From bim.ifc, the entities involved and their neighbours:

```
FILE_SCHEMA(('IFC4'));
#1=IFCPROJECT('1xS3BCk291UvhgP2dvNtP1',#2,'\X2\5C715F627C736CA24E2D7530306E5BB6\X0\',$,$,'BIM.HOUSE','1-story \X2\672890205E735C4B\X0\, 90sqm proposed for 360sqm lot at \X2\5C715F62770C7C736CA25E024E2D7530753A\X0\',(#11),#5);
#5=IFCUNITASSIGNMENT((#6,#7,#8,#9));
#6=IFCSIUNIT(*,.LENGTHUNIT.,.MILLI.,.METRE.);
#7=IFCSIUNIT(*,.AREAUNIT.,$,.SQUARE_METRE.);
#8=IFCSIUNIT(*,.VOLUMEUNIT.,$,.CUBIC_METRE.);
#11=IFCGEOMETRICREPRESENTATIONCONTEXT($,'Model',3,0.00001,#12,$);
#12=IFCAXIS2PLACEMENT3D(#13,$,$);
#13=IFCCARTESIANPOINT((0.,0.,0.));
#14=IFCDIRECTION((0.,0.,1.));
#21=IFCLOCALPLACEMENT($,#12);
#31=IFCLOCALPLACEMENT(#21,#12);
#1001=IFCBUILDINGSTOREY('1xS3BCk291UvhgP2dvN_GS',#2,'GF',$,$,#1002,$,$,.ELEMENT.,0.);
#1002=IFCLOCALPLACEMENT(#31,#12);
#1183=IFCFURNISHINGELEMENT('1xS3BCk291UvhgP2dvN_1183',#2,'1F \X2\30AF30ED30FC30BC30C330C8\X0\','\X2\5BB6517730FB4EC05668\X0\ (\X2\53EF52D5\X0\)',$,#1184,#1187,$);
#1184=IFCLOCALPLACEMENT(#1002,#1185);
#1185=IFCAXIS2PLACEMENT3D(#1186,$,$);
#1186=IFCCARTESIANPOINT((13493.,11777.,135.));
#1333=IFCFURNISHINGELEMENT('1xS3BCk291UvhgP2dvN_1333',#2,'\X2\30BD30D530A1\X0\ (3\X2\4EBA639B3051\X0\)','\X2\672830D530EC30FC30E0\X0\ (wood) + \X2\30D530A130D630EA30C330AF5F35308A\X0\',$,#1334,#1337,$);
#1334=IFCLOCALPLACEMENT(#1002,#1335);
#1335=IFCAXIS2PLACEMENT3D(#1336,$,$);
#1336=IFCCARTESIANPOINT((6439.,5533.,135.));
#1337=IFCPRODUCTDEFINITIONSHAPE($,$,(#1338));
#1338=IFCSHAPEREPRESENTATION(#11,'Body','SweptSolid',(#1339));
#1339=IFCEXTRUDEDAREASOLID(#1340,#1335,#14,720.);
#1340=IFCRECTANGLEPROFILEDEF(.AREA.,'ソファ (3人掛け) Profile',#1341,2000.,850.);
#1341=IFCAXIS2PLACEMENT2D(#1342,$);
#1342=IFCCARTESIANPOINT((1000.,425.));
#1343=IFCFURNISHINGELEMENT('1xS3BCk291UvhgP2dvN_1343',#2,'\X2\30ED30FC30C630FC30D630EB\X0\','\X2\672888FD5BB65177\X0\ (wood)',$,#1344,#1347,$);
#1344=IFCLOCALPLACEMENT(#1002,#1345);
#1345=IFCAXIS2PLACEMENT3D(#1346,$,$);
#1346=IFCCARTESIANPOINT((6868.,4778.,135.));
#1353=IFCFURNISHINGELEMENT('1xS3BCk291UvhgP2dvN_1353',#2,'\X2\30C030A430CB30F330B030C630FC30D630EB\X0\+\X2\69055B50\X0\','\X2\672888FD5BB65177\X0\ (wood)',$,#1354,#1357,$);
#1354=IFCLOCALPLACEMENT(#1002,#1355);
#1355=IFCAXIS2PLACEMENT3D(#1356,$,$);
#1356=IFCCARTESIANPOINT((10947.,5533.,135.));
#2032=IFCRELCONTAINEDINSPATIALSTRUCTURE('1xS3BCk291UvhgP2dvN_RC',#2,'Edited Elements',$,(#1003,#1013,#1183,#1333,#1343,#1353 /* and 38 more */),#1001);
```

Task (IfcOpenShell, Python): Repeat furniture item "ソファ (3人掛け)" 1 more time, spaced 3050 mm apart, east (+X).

```python
import numpy as np
import ifcopenshell
import ifcopenshell.api.geometry
import ifcopenshell.api.root
import ifcopenshell.util.element
import ifcopenshell.util.placement
import ifcopenshell.util.unit

model = ifcopenshell.open("bim.ifc")
unit_scale = ifcopenshell.util.unit.calculate_unit_scale(model)


def reuse_history(source, copy):
    """copy_class also copies each property set's owner history, people and application; keep the originals."""
    for rel in copy.IsDefinedBy:
        if rel.is_a("IfcRelDefinesByProperties") and (history := rel.RelatingPropertyDefinition.OwnerHistory):
            rel.RelatingPropertyDefinition.OwnerHistory = source.OwnerHistory
            ifcopenshell.util.element.remove_deep2(model, history)


source = model.by_guid("1xS3BCk291UvhgP2dvN_1333")
base = ifcopenshell.util.placement.get_local_placement(source.ObjectPlacement)
step = np.array([1.0, 0.0, 0.0]) * 3.05 / unit_scale

for i in range(1, 2):
    copy = ifcopenshell.api.root.copy_class(model, product=source)
    copy.Representation = ifcopenshell.util.element.copy_deep(
        model, source.Representation, exclude=["IfcGeometricRepresentationContext", "IfcRepresentationMap"]
    )
    reuse_history(source, copy)
    matrix = base.copy()
    matrix[:3, 3] += i * step
    print("added at", matrix[:3, 3].round(3) + 0.0)
    ifcopenshell.api.geometry.edit_object_placement(model, product=copy, matrix=matrix, is_si=False)

model.write("bim-out.ifc")
```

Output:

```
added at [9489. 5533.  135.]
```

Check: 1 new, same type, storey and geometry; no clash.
